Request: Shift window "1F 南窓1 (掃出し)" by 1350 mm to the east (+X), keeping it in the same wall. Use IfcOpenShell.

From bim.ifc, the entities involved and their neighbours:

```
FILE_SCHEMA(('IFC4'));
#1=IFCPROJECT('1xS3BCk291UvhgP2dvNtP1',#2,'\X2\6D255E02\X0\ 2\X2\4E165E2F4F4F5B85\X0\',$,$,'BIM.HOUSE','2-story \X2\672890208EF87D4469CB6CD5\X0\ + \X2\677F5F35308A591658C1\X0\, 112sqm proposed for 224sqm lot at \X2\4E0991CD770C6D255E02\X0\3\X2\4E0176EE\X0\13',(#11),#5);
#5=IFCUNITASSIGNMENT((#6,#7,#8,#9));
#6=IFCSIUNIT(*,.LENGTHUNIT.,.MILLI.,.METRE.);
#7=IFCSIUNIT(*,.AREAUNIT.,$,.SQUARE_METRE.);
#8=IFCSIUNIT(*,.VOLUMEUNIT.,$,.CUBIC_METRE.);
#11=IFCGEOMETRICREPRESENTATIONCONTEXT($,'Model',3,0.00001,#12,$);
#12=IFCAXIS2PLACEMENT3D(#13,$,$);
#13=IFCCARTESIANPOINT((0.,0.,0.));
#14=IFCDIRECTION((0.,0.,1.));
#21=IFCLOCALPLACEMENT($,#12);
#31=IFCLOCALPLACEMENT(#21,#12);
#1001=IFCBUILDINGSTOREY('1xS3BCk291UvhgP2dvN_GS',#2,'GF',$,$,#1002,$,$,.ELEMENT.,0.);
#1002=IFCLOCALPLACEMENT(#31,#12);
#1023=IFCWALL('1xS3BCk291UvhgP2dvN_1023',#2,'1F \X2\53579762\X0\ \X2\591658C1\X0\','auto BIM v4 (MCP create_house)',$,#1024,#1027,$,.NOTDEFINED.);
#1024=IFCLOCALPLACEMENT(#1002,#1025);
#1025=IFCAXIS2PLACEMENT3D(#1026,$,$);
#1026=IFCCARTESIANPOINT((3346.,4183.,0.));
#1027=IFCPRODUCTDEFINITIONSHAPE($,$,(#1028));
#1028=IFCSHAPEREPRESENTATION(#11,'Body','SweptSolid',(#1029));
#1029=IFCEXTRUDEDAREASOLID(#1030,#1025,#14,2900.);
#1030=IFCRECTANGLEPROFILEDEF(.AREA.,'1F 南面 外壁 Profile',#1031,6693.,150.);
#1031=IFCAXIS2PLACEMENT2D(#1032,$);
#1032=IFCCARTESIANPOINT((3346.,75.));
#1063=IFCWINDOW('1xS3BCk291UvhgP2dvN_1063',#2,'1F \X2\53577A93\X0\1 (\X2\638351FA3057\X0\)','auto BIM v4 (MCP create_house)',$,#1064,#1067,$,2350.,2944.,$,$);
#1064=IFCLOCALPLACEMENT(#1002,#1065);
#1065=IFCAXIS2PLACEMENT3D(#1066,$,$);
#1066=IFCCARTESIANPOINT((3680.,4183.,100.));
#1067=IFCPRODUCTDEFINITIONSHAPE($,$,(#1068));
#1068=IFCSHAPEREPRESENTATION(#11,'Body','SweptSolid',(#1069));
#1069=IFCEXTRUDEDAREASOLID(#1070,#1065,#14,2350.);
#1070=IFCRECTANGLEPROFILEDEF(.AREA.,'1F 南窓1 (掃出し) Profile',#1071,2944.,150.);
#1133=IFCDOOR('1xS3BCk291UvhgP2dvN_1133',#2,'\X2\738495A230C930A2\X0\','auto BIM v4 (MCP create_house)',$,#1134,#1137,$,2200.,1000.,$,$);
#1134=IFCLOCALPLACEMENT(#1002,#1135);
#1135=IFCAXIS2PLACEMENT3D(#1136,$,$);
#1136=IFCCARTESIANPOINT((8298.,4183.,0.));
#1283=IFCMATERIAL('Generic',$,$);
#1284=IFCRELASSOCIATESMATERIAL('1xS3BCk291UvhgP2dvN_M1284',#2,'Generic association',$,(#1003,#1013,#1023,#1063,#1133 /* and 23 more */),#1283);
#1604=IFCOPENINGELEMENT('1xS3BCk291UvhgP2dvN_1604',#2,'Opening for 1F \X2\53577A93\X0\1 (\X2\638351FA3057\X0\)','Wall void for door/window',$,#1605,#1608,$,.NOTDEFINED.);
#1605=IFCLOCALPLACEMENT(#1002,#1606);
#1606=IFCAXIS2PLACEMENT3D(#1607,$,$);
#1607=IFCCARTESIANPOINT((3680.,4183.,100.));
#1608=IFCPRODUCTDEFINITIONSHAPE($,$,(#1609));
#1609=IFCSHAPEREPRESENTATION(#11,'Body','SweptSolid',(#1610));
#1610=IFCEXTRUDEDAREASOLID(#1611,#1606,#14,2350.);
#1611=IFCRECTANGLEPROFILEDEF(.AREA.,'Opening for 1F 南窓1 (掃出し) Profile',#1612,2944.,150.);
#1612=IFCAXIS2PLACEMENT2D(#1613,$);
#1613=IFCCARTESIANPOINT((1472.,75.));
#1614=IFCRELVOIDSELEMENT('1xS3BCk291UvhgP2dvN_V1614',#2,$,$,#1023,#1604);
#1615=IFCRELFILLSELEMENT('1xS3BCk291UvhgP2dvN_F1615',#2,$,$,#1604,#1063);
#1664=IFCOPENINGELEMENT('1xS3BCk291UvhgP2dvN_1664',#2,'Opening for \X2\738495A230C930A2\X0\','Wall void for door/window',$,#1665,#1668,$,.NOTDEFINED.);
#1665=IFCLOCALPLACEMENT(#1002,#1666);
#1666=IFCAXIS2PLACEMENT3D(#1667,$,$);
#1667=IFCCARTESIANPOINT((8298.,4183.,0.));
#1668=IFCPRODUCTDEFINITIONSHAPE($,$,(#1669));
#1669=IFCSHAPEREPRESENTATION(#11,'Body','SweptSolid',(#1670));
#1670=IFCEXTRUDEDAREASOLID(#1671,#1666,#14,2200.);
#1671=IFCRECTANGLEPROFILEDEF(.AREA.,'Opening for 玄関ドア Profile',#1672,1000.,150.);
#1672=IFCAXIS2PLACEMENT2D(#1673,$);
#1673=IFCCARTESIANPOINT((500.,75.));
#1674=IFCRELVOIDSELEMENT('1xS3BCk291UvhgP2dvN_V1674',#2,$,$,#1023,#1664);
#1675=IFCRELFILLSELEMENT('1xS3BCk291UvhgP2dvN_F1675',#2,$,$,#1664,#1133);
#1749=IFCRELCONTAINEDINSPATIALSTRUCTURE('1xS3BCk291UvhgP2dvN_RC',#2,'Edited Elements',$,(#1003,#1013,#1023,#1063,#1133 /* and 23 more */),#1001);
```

```python
import ifcopenshell
import ifcopenshell.api.geometry
import ifcopenshell.util.placement
import ifcopenshell.util.unit

model = ifcopenshell.open("bim.ifc")
unit_scale = ifcopenshell.util.unit.calculate_unit_scale(model)

window = model.by_id(1063)
opening = window.FillsVoids[0].RelatingOpeningElement
wall = opening.VoidsElements[0].RelatingBuildingElement

wall_matrix = ifcopenshell.util.placement.get_local_placement(wall.ObjectPlacement)
shift = wall_matrix[:3, 0] * 1.35 / unit_scale
before = ifcopenshell.util.placement.get_local_placement(window.ObjectPlacement)[:3, 3].copy()

# The window is not placed relative to its opening, so move both.
for product in (opening, window):
    matrix = ifcopenshell.util.placement.get_local_placement(product.ObjectPlacement)
    matrix[:3, 3] += shift
    ifcopenshell.api.geometry.edit_object_placement(model, product=product, matrix=matrix, is_si=False)

after = ifcopenshell.util.placement.get_local_placement(window.ObjectPlacement)[:3, 3]
print("window moved by", (after - before).round(3) + 0.0)

model.write("bim_updated.ifc")
```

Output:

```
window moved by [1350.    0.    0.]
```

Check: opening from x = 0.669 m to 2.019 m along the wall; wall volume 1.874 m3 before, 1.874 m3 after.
